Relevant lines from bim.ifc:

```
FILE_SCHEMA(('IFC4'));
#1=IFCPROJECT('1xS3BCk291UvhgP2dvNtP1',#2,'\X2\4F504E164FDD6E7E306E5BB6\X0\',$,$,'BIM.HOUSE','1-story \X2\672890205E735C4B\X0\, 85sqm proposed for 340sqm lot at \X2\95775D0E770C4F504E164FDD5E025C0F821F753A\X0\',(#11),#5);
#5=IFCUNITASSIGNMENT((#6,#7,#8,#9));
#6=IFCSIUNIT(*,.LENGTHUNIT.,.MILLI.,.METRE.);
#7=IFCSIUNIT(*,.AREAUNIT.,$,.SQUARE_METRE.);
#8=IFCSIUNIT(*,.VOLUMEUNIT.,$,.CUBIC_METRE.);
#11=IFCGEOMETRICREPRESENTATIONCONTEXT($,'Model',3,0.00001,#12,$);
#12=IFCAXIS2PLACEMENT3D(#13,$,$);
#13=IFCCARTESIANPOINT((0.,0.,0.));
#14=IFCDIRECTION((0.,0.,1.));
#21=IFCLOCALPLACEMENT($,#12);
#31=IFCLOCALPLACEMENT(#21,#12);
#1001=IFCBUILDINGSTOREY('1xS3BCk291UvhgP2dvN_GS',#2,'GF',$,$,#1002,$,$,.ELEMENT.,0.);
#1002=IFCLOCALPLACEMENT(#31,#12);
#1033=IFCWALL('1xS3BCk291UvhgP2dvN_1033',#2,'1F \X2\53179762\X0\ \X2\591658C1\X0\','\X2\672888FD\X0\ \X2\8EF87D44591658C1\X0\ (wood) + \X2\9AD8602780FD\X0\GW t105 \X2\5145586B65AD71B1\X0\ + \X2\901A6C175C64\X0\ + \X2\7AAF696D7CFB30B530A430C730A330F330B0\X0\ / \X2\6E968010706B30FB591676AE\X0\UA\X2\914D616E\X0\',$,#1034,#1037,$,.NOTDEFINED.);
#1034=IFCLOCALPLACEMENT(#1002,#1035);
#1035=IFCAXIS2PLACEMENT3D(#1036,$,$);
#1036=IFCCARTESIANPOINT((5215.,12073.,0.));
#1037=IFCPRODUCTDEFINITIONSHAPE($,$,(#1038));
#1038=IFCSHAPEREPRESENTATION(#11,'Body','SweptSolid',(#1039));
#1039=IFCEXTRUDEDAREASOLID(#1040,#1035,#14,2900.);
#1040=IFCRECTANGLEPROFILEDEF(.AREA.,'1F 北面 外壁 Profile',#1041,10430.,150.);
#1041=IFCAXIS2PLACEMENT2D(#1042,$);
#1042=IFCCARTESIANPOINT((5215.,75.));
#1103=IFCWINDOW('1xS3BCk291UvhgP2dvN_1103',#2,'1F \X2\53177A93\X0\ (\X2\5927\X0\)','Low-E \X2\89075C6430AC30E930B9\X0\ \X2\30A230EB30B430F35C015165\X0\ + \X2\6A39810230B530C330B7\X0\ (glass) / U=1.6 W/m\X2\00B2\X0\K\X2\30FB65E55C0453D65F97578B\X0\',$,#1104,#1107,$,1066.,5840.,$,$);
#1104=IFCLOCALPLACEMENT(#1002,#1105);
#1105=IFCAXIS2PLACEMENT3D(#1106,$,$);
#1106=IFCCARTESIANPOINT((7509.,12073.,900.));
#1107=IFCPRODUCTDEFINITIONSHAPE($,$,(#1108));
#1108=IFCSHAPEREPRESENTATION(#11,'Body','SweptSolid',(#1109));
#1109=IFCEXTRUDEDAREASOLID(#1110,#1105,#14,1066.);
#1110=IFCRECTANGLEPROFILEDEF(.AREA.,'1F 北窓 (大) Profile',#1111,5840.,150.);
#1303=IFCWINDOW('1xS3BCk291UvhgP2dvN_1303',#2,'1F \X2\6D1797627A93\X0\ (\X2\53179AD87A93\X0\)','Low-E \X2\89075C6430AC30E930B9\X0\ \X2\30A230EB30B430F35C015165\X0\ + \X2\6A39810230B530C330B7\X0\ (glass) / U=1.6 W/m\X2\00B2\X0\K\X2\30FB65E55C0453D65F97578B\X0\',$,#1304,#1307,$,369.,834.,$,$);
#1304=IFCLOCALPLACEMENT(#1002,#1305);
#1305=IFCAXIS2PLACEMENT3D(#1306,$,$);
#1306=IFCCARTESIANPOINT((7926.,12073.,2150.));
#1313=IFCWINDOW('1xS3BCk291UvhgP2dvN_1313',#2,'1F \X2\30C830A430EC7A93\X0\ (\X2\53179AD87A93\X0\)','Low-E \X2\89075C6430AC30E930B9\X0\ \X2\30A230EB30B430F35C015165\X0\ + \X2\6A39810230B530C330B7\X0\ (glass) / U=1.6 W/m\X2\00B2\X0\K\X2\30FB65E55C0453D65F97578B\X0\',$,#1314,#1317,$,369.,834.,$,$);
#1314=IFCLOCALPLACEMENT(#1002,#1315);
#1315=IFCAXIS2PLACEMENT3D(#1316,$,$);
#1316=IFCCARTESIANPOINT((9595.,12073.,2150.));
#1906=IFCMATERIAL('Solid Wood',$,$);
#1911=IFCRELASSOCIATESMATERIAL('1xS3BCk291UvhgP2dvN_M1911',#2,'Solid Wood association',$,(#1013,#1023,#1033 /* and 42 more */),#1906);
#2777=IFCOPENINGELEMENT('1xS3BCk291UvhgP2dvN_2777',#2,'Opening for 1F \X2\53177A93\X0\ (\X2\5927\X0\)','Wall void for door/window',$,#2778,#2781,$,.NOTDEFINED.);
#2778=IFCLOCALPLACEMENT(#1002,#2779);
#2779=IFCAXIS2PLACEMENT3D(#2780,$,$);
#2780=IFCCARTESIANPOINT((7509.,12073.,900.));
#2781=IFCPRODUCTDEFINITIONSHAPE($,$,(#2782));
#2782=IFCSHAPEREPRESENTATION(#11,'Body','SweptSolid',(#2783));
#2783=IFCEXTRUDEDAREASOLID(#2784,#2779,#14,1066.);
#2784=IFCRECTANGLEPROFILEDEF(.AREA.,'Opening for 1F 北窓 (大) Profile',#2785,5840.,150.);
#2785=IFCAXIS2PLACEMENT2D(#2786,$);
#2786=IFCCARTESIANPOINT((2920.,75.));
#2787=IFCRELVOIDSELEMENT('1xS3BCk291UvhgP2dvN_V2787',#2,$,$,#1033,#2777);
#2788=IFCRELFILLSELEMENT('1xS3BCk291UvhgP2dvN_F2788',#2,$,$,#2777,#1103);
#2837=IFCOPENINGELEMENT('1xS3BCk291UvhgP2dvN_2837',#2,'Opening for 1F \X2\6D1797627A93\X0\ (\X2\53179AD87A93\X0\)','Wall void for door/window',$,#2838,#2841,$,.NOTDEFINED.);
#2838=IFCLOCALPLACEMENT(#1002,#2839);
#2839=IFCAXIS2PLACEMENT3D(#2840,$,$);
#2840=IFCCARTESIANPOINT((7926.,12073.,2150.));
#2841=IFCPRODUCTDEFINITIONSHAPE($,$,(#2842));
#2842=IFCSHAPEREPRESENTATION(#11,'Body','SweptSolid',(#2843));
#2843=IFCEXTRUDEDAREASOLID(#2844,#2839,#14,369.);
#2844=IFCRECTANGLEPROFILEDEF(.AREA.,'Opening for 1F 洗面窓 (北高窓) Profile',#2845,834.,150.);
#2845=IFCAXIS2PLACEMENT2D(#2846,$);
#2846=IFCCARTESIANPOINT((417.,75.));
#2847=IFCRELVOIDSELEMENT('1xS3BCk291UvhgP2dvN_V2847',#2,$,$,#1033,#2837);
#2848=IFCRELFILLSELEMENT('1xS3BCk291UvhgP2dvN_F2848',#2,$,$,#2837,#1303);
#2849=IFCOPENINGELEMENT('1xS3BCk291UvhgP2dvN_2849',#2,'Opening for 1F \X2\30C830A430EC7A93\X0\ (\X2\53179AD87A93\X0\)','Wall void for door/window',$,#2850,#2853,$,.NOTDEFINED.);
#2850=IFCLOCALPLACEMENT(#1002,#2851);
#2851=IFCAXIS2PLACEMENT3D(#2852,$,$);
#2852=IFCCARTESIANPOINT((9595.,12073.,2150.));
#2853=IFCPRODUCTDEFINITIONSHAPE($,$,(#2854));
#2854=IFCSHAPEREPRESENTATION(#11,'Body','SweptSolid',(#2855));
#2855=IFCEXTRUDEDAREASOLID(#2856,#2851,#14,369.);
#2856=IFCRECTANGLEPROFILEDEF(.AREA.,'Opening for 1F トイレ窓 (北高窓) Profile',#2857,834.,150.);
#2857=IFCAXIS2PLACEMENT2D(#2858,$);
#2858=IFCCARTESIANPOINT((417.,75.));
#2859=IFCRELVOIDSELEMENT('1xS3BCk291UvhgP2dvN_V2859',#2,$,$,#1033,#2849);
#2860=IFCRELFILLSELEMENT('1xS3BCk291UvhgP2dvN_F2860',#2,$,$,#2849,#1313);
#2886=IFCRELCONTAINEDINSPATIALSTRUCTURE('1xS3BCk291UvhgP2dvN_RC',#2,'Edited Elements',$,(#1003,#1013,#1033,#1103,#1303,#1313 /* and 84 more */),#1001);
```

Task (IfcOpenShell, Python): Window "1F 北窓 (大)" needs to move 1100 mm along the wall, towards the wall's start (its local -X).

```python
import ifcopenshell
import ifcopenshell.api.geometry
import ifcopenshell.util.placement

model = ifcopenshell.open("bim.ifc")

window = model.by_guid("1xS3BCk291UvhgP2dvN_1103")
opening = window.FillsVoids[0].RelatingOpeningElement
wall = opening.VoidsElements[0].RelatingBuildingElement

wall_matrix = ifcopenshell.util.placement.get_local_placement(wall.ObjectPlacement)
shift = wall_matrix[:3, 0] * -1100.0
before = ifcopenshell.util.placement.get_local_placement(window.ObjectPlacement)[:3, 3].copy()

# The window is not placed relative to its opening, so move both.
for product in (opening, window):
    matrix = ifcopenshell.util.placement.get_local_placement(product.ObjectPlacement)
    matrix[:3, 3] += shift
    ifcopenshell.api.geometry.edit_object_placement(model, product=product, matrix=matrix, is_si=False)

after = ifcopenshell.util.placement.get_local_placement(window.ObjectPlacement)[:3, 3]
print("window moved by", (after - before).round(3) + 0.0)

model.write("bim_rev.ifc")
```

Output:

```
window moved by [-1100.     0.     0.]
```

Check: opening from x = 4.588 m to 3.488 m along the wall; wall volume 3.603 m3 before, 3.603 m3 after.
